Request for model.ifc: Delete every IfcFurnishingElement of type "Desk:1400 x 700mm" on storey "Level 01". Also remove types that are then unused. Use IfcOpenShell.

First a look at what the model holds.

```python
import ifcopenshell
import ifcopenshell.util.element

model = ifcopenshell.open("model.ifc")
print(model.schema)
storey = next(s for s in model.by_type("IfcBuildingStorey") if s.Name == "Level 01")
furniture = [e for e in ifcopenshell.util.element.get_decomposition(storey) if e.is_a("IfcFurnishingElement")]
seen = {}
for e in furniture:
    element_type = ifcopenshell.util.element.get_type(e)
    name = element_type.Name if element_type not in (None, e) else None
    seen[name] = seen.get(name, 0) + 1
for name, count in sorted(seen.items(), key=str):
    print(count, "x", name)
```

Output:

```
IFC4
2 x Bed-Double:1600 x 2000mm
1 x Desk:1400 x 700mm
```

```python
import ifcopenshell
import ifcopenshell.api.root
import ifcopenshell.util.element

model = ifcopenshell.open("model.ifc")

storey = next(s for s in model.by_type("IfcBuildingStorey") if s.Name == "Level 01")
furniture = [e for e in ifcopenshell.util.element.get_decomposition(storey) if e.is_a("IfcFurnishingElement")]
targets = [e for e in furniture if (t := ifcopenshell.util.element.get_type(e)) not in (None, e) and t.Name == "Desk:1400 x 700mm"]
types = {ifcopenshell.util.element.get_type(e) for e in targets} - {None, *targets}

for e in targets:
    ifcopenshell.api.root.remove_product(model, product=e)
print(len(targets), "removed")

unused = [t for t in types if not ifcopenshell.util.element.get_types(t)]
for t in unused:
    ifcopenshell.api.root.remove_product(model, product=t)
print(len(unused), "unused types removed")

model.write("model_rev.ifc")
```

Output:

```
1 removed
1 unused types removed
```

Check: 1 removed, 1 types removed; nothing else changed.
